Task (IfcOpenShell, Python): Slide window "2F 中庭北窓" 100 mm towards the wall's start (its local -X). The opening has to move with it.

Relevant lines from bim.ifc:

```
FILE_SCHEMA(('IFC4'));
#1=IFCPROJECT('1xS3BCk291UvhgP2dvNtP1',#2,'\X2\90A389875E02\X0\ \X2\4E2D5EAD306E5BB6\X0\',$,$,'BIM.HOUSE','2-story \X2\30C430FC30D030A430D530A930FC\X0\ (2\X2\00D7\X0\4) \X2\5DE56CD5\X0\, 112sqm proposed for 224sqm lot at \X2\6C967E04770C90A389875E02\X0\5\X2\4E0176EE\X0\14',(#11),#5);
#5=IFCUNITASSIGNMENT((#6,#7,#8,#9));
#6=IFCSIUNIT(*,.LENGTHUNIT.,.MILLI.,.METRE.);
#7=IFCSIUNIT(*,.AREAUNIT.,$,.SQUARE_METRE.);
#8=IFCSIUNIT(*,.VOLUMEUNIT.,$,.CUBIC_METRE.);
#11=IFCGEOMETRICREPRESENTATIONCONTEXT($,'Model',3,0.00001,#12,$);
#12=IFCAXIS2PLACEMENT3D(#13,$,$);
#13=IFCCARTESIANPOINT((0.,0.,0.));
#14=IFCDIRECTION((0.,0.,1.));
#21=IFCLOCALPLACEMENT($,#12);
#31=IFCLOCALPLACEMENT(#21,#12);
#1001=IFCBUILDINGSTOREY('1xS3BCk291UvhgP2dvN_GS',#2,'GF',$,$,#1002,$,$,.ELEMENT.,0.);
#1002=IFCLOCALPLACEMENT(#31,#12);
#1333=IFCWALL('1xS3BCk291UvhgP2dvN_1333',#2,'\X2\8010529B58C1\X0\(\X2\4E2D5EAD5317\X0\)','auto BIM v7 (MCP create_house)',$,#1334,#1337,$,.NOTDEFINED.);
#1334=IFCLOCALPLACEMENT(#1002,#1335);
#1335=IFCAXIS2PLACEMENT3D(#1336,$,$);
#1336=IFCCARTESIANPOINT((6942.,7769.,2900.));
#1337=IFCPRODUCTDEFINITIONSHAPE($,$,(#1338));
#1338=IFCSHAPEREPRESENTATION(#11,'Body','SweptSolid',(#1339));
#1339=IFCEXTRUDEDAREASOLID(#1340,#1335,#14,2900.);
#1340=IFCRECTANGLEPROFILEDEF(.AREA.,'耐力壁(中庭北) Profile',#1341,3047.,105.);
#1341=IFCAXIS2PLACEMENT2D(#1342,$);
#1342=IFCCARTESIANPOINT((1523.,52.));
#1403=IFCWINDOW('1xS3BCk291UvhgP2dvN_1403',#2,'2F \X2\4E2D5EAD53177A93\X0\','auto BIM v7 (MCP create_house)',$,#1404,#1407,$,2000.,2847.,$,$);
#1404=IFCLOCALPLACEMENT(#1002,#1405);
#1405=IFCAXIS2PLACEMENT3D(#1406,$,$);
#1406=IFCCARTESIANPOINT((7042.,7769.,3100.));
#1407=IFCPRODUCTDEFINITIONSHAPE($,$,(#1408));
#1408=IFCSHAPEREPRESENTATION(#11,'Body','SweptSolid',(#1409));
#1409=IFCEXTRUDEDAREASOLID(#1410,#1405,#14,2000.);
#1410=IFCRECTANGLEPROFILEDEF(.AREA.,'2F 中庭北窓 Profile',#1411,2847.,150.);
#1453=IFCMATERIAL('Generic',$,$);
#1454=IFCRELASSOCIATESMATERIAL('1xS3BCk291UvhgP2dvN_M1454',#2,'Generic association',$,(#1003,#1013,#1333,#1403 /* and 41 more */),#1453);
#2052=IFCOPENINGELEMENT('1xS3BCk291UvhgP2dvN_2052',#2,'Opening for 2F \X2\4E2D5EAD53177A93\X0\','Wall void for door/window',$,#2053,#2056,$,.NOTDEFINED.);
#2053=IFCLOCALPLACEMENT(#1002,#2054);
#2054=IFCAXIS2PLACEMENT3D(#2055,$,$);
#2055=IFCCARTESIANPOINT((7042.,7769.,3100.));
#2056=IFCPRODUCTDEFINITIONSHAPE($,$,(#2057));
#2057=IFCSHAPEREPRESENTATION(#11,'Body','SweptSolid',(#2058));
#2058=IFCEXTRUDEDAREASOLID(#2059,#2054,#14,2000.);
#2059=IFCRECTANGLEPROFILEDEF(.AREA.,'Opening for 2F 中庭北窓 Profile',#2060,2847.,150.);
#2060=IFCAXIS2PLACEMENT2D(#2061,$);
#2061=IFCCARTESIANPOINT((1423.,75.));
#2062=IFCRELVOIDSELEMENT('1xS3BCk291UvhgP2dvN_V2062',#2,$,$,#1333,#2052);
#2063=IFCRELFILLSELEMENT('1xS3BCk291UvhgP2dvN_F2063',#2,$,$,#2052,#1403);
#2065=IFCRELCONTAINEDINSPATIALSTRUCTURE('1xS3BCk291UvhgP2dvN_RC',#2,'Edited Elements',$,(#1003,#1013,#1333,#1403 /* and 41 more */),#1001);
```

```python
import ifcopenshell
import ifcopenshell.api.geometry
import ifcopenshell.util.placement

model = ifcopenshell.open("bim.ifc")

window = model.by_guid("1xS3BCk291UvhgP2dvN_1403")
opening = window.FillsVoids[0].RelatingOpeningElement
wall = opening.VoidsElements[0].RelatingBuildingElement

wall_matrix = ifcopenshell.util.placement.get_local_placement(wall.ObjectPlacement)
shift = wall_matrix[:3, 0] * -100.0
before = ifcopenshell.util.placement.get_local_placement(window.ObjectPlacement)[:3, 3].copy()

# The window is not placed relative to its opening, so move both.
for product in (opening, window):
    matrix = ifcopenshell.util.placement.get_local_placement(product.ObjectPlacement)
    matrix[:3, 3] += shift
    ifcopenshell.api.geometry.edit_object_placement(model, product=product, matrix=matrix, is_si=False)

after = ifcopenshell.util.placement.get_local_placement(window.ObjectPlacement)[:3, 3]
print("window moved by", (after - before).round(3) + 0.0)

model.write("bim-out.ifc")
```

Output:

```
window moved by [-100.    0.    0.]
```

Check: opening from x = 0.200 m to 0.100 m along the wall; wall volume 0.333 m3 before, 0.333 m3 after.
